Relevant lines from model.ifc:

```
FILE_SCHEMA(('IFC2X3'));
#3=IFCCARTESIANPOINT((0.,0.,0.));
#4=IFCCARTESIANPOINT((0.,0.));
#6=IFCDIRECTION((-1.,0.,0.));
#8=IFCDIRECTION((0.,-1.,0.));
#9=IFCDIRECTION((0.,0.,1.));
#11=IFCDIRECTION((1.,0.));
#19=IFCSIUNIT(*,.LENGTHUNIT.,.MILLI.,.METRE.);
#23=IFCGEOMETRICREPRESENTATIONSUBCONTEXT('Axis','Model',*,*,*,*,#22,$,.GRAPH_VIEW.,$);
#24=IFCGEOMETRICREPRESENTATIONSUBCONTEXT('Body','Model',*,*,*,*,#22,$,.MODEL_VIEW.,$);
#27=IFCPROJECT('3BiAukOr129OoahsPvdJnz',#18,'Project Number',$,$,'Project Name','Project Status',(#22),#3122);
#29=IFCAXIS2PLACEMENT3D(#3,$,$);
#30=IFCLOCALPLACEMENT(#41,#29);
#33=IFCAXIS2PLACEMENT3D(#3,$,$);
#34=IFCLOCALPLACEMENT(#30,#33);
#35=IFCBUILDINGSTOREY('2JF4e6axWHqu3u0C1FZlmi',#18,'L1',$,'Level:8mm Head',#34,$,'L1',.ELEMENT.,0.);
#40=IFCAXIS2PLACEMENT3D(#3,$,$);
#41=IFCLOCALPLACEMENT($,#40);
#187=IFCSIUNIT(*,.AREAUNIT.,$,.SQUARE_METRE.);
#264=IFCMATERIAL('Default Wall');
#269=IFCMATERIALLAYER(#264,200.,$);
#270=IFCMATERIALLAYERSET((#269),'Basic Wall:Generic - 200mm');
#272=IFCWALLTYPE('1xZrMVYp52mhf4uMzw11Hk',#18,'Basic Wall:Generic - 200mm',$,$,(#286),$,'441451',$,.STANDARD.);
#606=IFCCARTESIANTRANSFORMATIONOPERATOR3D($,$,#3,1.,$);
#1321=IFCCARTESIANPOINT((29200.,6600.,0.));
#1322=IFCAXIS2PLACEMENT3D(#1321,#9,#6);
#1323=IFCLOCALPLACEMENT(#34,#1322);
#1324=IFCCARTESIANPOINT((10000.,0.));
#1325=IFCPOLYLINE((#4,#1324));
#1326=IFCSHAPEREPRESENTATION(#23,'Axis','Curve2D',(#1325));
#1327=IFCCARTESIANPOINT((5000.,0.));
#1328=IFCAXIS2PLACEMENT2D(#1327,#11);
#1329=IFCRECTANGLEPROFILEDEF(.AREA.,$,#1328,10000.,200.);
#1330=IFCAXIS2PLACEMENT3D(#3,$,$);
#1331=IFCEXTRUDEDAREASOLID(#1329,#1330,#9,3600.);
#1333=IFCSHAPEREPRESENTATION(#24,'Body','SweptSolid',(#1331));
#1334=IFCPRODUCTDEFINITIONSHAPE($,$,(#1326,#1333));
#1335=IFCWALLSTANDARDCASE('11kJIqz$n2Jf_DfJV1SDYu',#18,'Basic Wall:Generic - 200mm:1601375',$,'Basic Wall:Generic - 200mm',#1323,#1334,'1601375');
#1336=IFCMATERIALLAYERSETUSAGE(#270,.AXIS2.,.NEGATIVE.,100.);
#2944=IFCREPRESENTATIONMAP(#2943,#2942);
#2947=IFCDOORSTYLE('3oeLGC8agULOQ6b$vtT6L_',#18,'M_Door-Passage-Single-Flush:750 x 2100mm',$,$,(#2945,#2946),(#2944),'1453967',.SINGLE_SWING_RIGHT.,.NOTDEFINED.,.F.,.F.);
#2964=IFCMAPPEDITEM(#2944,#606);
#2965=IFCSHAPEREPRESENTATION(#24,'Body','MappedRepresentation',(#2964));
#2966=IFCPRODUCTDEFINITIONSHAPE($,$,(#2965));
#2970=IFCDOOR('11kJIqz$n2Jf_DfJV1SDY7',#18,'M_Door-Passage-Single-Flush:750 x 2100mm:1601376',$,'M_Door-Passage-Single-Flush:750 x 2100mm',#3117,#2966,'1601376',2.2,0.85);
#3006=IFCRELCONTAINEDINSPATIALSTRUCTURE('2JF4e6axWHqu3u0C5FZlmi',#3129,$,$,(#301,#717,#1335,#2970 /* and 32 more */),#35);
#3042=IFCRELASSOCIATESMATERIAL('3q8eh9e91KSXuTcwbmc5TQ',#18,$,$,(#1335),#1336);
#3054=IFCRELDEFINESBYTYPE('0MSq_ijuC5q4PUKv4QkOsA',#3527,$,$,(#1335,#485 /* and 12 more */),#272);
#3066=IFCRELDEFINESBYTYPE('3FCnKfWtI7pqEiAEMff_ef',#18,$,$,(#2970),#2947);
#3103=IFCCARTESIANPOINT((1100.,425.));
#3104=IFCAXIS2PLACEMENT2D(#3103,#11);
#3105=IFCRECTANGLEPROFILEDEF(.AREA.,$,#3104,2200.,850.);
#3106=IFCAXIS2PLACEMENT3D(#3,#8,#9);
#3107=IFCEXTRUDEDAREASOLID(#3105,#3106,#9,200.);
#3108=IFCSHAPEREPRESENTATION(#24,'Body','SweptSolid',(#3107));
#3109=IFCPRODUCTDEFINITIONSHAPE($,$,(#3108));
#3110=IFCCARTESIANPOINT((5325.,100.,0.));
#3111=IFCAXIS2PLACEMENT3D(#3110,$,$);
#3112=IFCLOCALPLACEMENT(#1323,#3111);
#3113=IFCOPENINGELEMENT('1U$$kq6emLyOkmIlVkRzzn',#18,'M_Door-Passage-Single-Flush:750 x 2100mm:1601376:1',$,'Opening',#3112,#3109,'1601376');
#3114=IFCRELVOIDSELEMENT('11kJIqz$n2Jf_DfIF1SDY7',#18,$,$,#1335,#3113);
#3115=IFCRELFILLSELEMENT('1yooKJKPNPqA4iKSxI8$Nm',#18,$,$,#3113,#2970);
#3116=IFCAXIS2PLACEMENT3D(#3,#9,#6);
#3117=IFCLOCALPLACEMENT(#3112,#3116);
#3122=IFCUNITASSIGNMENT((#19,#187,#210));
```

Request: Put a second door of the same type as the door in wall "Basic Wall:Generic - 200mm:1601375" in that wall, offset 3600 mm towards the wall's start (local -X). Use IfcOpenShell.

```python
import ifcopenshell
import ifcopenshell.api.feature
import ifcopenshell.api.geometry
import ifcopenshell.api.root
import ifcopenshell.geom
import ifcopenshell.util.element
import ifcopenshell.util.placement
import ifcopenshell.util.shape
import ifcopenshell.util.unit

model = ifcopenshell.open("model.ifc")
unit_scale = ifcopenshell.util.unit.calculate_unit_scale(model)
settings = ifcopenshell.geom.settings()


def volume(element):
    """Net volume in cubic metres, openings subtracted."""
    shape = ifcopenshell.geom.create_shape(settings, element)
    return ifcopenshell.util.shape.get_volume(shape.geometry)


def reuse_history(source, copy):
    """copy_class also copies each property set's owner history, people and application; keep the originals."""
    for rel in copy.IsDefinedBy:
        if rel.is_a("IfcRelDefinesByProperties") and (history := rel.RelatingPropertyDefinition.OwnerHistory):
            rel.RelatingPropertyDefinition.OwnerHistory = source.OwnerHistory
            ifcopenshell.util.element.remove_deep2(model, history)


door = model.by_id(2970)
opening = door.FillsVoids[0].RelatingOpeningElement
wall = opening.VoidsElements[0].RelatingBuildingElement
before = volume(wall)
shift = ifcopenshell.util.placement.get_local_placement(wall.ObjectPlacement)[:3, 0] * -3.6 / unit_scale

# copy_class copies the void relationship, type, container and properties, but no geometry.
new_opening = ifcopenshell.api.root.copy_class(model, product=opening)
new_opening.Representation = ifcopenshell.util.element.copy_deep(
    model, opening.Representation, exclude=["IfcGeometricRepresentationContext", "IfcRepresentationMap"]
)
new_opening.Name = "M_Door-Passage-Single-Flush:750 x 2100mm"
new_opening.Tag = None
new_door = ifcopenshell.api.root.copy_class(model, product=door)
new_door.Representation = ifcopenshell.util.element.copy_deep(
    model, door.Representation, exclude=["IfcGeometricRepresentationContext", "IfcRepresentationMap"]
)
new_door.Name = "M_Door-Passage-Single-Flush:750 x 2100mm"
new_door.Tag = None
reuse_history(door, new_door)
fills = ifcopenshell.api.feature.add_filling(model, opening=new_opening, element=new_door)
fills.OwnerHistory = new_door.OwnerHistory  # required in IFC2X3

for old, new in ((opening, new_opening), (door, new_door)):
    matrix = ifcopenshell.util.placement.get_local_placement(old.ObjectPlacement)
    matrix[:3, 3] += shift
    ifcopenshell.api.geometry.edit_object_placement(model, product=new, matrix=matrix, is_si=False)

after = volume(wall)

print(f"wall volume {before:.3f} -> {after:.3f} m3")

model.write("model_updated.ifc")
```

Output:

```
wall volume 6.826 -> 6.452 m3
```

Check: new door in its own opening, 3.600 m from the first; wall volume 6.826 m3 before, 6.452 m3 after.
